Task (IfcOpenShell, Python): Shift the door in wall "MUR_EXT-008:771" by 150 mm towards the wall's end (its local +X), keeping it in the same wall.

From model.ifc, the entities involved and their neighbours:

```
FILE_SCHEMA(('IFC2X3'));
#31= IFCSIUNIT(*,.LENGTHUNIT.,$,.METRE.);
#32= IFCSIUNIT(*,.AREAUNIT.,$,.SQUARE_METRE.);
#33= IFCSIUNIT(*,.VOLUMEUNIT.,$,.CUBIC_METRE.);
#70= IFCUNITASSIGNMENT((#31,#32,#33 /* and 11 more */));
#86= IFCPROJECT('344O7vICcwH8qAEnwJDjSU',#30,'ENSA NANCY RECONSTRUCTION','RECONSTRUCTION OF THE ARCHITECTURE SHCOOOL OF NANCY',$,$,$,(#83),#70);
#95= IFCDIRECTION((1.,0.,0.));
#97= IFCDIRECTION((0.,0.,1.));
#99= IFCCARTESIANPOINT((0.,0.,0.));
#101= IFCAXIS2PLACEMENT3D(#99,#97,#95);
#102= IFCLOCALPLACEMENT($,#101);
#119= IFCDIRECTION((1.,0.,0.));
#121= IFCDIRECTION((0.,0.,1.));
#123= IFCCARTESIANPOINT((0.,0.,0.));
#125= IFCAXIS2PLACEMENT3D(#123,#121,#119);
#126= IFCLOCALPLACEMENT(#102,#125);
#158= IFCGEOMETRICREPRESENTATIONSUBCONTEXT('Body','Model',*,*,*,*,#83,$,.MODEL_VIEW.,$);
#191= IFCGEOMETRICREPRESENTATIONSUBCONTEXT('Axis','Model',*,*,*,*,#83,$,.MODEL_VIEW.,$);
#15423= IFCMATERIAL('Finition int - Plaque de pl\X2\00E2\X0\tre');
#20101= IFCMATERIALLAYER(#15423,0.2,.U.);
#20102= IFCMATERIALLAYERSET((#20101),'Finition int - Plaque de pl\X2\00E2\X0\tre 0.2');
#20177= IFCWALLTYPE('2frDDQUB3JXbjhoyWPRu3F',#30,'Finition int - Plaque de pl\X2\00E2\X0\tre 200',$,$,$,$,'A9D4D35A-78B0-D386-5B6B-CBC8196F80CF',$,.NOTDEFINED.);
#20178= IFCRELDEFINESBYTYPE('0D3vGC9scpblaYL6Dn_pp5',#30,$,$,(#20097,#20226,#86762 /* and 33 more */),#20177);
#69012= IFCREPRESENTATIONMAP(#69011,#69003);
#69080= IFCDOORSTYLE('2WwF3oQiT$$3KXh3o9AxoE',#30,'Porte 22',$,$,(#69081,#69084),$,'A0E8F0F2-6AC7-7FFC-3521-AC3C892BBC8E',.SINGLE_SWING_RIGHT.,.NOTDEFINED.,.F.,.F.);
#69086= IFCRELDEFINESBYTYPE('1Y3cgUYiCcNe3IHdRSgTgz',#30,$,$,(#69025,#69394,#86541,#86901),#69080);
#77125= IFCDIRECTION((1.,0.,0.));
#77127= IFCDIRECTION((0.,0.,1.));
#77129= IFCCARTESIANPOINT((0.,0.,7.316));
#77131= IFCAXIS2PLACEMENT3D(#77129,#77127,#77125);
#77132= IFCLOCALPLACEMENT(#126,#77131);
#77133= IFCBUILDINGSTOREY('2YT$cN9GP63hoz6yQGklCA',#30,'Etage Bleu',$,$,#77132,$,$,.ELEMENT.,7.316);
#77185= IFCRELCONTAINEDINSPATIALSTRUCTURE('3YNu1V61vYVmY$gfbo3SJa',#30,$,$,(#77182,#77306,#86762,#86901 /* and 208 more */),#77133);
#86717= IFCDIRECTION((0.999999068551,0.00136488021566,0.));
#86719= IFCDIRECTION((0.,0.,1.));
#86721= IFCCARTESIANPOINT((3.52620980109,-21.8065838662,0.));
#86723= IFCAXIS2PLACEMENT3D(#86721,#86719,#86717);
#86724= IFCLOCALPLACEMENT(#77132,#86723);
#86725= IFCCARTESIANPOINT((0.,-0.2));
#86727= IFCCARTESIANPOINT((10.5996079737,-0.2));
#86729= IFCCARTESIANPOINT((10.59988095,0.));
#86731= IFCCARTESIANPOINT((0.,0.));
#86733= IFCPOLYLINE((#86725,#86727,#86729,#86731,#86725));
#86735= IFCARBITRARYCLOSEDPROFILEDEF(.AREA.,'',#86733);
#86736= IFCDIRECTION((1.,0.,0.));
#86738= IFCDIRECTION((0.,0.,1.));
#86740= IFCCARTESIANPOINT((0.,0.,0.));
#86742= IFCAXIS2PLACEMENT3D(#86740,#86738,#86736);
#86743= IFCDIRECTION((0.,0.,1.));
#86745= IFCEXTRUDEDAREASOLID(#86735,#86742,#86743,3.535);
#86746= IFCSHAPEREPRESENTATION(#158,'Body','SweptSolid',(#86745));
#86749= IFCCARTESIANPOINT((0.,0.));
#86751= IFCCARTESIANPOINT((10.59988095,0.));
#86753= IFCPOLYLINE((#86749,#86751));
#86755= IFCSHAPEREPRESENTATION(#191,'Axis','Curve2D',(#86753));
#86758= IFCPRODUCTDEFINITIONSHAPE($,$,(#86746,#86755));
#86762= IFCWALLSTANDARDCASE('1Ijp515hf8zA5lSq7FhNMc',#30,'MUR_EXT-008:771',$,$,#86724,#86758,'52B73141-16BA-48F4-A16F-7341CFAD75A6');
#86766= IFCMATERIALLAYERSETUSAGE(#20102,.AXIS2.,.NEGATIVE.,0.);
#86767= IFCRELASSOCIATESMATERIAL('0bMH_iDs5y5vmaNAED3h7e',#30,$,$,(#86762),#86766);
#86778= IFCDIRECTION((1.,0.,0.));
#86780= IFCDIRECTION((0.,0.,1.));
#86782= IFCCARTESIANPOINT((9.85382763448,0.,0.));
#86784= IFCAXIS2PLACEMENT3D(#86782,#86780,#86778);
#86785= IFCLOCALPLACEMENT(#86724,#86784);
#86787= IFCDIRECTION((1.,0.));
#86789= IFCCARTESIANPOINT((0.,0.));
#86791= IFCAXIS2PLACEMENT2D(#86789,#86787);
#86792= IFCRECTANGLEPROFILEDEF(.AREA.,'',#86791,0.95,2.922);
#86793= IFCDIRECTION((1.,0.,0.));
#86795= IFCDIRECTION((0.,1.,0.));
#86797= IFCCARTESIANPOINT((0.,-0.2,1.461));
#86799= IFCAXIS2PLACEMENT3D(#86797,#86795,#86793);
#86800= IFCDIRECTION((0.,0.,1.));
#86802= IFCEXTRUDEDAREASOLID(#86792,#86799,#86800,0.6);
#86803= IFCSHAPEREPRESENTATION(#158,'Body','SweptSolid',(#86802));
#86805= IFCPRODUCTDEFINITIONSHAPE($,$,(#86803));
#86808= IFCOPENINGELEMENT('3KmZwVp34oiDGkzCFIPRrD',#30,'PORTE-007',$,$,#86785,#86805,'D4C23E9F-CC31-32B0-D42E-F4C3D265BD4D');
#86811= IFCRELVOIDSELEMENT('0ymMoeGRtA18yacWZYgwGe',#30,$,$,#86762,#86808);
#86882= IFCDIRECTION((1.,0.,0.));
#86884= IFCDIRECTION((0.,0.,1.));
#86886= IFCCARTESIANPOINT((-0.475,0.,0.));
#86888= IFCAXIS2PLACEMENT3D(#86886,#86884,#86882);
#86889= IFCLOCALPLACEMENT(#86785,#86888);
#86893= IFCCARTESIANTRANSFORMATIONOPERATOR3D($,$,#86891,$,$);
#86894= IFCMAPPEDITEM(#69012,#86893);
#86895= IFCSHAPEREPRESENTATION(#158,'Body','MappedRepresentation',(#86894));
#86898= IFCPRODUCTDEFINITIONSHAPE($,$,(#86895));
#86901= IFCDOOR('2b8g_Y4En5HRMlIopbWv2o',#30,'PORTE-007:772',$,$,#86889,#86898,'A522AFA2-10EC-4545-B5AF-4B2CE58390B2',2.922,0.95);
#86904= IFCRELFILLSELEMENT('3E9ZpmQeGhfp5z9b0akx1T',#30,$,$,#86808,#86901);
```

```python
import ifcopenshell
import ifcopenshell.api.geometry
import ifcopenshell.util.placement
import ifcopenshell.util.unit

model = ifcopenshell.open("model.ifc")
unit_scale = ifcopenshell.util.unit.calculate_unit_scale(model)

door = model.by_guid("2b8g_Y4En5HRMlIopbWv2o")
opening = door.FillsVoids[0].RelatingOpeningElement
wall = opening.VoidsElements[0].RelatingBuildingElement

wall_matrix = ifcopenshell.util.placement.get_local_placement(wall.ObjectPlacement)
shift = wall_matrix[:3, 0] * 0.15 / unit_scale
before = ifcopenshell.util.placement.get_local_placement(door.ObjectPlacement)[:3, 3].copy()

# The door is placed relative to its opening, so it follows when the opening moves.
matrix = ifcopenshell.util.placement.get_local_placement(opening.ObjectPlacement)
matrix[:3, 3] += shift
ifcopenshell.api.geometry.edit_object_placement(
    model, product=opening, matrix=matrix, is_si=False, should_transform_children=True
)

after = ifcopenshell.util.placement.get_local_placement(door.ObjectPlacement)[:3, 3]
print("door moved by", (after - before).round(3) + 0.0)

model.write("model_rev.ifc")
```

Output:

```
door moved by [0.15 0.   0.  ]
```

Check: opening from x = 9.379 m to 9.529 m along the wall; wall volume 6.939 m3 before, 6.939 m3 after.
